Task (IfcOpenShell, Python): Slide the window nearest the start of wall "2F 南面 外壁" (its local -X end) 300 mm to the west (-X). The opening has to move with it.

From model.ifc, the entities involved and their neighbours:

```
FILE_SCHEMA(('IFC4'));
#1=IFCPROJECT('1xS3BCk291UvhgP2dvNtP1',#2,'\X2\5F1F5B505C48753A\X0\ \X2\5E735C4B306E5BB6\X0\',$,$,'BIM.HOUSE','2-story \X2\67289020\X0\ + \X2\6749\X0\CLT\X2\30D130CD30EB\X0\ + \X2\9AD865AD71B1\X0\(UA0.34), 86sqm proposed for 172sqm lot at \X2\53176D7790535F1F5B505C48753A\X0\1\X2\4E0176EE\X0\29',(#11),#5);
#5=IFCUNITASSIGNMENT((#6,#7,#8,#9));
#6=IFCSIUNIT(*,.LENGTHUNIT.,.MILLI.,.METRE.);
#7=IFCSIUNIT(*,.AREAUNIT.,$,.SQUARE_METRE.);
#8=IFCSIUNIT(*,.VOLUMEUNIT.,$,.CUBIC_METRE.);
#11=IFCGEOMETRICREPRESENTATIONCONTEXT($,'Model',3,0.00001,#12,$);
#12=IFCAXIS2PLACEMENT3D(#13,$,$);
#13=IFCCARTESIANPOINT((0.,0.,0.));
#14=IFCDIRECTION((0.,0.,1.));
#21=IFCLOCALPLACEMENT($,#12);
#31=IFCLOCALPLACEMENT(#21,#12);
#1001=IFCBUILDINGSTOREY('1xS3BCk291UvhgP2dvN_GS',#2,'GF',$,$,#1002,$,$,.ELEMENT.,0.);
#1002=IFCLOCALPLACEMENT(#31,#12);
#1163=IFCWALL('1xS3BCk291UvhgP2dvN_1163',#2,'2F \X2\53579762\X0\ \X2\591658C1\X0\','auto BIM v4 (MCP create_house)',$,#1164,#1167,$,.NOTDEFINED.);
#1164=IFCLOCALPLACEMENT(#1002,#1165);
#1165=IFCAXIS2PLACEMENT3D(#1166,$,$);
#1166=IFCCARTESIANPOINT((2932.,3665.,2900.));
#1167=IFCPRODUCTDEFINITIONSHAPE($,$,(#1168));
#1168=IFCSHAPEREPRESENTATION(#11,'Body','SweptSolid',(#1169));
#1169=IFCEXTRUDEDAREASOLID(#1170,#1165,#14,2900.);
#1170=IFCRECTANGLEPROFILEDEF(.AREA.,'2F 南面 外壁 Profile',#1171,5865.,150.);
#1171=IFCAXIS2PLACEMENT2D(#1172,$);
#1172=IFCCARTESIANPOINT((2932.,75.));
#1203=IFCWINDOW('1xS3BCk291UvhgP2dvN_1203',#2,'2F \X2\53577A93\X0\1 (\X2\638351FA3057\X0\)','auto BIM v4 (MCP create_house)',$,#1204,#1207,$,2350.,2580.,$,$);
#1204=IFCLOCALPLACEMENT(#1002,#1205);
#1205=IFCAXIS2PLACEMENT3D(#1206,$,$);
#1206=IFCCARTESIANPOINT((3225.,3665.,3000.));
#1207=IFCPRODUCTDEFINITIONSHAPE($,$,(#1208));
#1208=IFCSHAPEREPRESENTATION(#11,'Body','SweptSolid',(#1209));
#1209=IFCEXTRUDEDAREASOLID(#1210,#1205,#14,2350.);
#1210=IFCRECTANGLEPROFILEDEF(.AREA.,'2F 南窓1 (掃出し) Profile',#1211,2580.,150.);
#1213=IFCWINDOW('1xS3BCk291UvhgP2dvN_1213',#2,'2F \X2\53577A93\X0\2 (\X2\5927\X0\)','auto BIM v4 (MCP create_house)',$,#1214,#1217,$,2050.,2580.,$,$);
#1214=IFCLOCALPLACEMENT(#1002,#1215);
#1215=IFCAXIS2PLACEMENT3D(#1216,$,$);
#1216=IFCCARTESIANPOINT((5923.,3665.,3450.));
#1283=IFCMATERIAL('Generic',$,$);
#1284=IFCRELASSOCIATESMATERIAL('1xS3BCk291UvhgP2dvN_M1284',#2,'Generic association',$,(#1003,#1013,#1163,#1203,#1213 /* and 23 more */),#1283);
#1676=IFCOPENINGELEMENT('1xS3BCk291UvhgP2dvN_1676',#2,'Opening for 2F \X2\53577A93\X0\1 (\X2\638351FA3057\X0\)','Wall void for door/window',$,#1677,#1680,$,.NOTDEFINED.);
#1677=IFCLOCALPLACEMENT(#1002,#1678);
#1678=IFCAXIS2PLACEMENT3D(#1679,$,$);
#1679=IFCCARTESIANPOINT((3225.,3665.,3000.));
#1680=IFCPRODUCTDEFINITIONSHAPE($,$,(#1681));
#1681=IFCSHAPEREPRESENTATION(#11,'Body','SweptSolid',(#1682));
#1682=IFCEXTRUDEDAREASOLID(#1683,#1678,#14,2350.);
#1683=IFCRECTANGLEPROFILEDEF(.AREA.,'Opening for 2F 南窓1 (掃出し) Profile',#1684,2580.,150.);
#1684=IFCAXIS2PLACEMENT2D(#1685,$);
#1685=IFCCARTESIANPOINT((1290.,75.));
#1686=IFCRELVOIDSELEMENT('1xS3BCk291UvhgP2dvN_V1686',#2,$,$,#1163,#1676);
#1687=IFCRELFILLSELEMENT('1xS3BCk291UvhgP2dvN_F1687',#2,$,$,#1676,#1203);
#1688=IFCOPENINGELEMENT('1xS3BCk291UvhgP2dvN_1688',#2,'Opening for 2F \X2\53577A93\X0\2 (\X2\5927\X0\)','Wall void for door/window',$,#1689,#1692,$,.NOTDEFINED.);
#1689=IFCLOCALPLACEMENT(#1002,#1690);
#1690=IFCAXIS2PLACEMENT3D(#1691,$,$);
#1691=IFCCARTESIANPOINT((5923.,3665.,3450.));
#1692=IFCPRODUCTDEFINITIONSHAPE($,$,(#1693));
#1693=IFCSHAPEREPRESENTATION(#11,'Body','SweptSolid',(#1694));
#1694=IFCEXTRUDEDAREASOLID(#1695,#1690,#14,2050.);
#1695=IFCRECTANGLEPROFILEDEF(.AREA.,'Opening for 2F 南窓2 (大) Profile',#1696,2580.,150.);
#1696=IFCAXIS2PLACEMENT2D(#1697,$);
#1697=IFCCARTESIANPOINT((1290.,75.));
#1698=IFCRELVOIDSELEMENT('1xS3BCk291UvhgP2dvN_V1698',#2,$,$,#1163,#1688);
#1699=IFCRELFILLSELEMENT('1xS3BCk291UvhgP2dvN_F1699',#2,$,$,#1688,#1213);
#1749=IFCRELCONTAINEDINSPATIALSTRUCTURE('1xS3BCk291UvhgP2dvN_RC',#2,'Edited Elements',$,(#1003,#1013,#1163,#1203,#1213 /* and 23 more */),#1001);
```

```python
import ifcopenshell
import ifcopenshell.api.geometry
import ifcopenshell.util.placement
import ifcopenshell.util.unit

model = ifcopenshell.open("model.ifc")
unit_scale = ifcopenshell.util.unit.calculate_unit_scale(model)

window = model.by_id(1203)
opening = window.FillsVoids[0].RelatingOpeningElement
wall = opening.VoidsElements[0].RelatingBuildingElement

wall_matrix = ifcopenshell.util.placement.get_local_placement(wall.ObjectPlacement)
shift = wall_matrix[:3, 0] * -0.3 / unit_scale
before = ifcopenshell.util.placement.get_local_placement(window.ObjectPlacement)[:3, 3].copy()

# The window is not placed relative to its opening, so move both.
for product in (opening, window):
    matrix = ifcopenshell.util.placement.get_local_placement(product.ObjectPlacement)
    matrix[:3, 3] += shift
    ifcopenshell.api.geometry.edit_object_placement(model, product=product, matrix=matrix, is_si=False)

after = ifcopenshell.util.placement.get_local_placement(window.ObjectPlacement)[:3, 3]
print("window moved by", (after - before).round(3) + 0.0)

model.write("model_edited.ifc")
```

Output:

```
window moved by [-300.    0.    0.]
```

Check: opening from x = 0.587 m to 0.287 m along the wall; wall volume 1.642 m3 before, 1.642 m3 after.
